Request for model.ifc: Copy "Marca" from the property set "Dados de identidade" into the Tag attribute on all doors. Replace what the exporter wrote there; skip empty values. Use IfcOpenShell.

First a look at what the model holds.

```python
import ifcopenshell
import ifcopenshell.util.element

model = ifcopenshell.open("model.ifc")
print(model.schema)
doors = model.by_type("IfcDoor")
print(len(doors), "doors")
for e in doors[:8]:
    source = ifcopenshell.util.element.get_pset(e, "Dados de identidade", "Marca")
    target = e.Tag
    print(e.id(), repr(source), repr(target), sep=" | ")
```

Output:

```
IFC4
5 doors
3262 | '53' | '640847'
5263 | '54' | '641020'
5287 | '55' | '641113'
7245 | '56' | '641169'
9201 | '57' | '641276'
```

```python
import ifcopenshell
import ifcopenshell.util.element

model = ifcopenshell.open("model.ifc")

count = 0
for e in model.by_type("IfcDoor"):
    value = ifcopenshell.util.element.get_pset(e, "Dados de identidade", "Marca")
    current = e.Tag
    if not value or not value.strip() or current == value:
        continue
    e.Tag = value
    count += 1

print(count, "doors updated")

model.write("model_rev.ifc")
```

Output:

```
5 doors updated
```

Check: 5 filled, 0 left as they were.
